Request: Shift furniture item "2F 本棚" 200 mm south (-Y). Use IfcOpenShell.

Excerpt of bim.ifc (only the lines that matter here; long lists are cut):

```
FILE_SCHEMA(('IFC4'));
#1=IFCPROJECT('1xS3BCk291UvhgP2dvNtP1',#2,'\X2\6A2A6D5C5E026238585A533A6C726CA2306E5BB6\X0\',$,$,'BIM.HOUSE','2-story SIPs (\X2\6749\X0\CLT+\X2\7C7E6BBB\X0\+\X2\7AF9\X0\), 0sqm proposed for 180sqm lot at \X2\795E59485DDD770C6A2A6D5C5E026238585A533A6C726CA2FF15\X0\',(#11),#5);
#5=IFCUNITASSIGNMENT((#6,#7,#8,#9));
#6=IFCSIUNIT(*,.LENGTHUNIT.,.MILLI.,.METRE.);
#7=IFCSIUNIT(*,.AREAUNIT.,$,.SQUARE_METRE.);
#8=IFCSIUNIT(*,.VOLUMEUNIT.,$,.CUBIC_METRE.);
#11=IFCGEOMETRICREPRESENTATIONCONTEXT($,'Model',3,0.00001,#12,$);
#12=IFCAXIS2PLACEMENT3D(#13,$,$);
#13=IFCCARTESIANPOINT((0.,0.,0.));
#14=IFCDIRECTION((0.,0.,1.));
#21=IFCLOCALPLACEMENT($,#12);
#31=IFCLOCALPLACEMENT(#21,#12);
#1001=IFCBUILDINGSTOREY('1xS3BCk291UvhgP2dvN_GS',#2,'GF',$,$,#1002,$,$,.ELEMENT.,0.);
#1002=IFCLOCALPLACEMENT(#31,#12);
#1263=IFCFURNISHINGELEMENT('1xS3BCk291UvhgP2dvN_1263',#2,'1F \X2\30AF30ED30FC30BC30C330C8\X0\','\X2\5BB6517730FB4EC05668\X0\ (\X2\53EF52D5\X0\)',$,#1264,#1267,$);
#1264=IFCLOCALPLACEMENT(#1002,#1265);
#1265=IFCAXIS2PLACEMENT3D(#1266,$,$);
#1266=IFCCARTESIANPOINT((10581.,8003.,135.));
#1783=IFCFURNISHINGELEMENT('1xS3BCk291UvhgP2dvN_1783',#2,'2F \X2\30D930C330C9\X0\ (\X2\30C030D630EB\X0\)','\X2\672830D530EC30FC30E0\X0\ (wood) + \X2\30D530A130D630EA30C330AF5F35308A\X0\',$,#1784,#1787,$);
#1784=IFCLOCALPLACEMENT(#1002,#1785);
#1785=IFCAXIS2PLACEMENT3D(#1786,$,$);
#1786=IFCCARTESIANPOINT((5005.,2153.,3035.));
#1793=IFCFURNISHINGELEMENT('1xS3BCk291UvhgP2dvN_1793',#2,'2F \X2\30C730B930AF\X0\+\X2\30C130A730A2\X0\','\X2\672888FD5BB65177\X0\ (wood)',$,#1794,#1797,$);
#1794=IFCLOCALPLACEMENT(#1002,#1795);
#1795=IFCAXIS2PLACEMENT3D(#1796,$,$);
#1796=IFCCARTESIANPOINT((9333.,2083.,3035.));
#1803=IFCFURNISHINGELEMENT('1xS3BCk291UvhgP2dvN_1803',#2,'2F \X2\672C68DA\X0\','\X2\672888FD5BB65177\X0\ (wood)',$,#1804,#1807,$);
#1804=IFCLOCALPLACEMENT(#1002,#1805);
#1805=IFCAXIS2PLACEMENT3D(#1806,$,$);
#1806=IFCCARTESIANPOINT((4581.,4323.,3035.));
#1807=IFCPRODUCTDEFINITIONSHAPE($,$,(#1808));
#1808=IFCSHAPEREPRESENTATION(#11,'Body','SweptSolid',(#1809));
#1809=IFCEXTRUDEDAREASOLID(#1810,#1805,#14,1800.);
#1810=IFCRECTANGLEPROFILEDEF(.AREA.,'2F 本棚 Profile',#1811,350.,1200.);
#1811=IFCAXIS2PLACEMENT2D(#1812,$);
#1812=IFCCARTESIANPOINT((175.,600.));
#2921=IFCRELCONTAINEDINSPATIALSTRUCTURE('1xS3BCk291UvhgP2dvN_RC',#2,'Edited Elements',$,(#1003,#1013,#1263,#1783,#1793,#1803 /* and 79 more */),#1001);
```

```python
import ifcopenshell
import ifcopenshell.api.geometry
import ifcopenshell.util.placement

model = ifcopenshell.open("bim.ifc")

item = model.by_guid("1xS3BCk291UvhgP2dvN_1803")
matrix = ifcopenshell.util.placement.get_local_placement(item.ObjectPlacement)
matrix[1, 3] -= 200.0
ifcopenshell.api.geometry.edit_object_placement(model, product=item, matrix=matrix, is_si=False)

print(ifcopenshell.util.placement.get_local_placement(item.ObjectPlacement).round(3) + 0.0)

model.write("bim_rev.ifc")
```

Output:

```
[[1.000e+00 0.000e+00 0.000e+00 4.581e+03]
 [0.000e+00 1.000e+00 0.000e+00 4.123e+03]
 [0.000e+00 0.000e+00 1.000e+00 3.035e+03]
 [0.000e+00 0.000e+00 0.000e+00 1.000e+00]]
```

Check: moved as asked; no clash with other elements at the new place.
